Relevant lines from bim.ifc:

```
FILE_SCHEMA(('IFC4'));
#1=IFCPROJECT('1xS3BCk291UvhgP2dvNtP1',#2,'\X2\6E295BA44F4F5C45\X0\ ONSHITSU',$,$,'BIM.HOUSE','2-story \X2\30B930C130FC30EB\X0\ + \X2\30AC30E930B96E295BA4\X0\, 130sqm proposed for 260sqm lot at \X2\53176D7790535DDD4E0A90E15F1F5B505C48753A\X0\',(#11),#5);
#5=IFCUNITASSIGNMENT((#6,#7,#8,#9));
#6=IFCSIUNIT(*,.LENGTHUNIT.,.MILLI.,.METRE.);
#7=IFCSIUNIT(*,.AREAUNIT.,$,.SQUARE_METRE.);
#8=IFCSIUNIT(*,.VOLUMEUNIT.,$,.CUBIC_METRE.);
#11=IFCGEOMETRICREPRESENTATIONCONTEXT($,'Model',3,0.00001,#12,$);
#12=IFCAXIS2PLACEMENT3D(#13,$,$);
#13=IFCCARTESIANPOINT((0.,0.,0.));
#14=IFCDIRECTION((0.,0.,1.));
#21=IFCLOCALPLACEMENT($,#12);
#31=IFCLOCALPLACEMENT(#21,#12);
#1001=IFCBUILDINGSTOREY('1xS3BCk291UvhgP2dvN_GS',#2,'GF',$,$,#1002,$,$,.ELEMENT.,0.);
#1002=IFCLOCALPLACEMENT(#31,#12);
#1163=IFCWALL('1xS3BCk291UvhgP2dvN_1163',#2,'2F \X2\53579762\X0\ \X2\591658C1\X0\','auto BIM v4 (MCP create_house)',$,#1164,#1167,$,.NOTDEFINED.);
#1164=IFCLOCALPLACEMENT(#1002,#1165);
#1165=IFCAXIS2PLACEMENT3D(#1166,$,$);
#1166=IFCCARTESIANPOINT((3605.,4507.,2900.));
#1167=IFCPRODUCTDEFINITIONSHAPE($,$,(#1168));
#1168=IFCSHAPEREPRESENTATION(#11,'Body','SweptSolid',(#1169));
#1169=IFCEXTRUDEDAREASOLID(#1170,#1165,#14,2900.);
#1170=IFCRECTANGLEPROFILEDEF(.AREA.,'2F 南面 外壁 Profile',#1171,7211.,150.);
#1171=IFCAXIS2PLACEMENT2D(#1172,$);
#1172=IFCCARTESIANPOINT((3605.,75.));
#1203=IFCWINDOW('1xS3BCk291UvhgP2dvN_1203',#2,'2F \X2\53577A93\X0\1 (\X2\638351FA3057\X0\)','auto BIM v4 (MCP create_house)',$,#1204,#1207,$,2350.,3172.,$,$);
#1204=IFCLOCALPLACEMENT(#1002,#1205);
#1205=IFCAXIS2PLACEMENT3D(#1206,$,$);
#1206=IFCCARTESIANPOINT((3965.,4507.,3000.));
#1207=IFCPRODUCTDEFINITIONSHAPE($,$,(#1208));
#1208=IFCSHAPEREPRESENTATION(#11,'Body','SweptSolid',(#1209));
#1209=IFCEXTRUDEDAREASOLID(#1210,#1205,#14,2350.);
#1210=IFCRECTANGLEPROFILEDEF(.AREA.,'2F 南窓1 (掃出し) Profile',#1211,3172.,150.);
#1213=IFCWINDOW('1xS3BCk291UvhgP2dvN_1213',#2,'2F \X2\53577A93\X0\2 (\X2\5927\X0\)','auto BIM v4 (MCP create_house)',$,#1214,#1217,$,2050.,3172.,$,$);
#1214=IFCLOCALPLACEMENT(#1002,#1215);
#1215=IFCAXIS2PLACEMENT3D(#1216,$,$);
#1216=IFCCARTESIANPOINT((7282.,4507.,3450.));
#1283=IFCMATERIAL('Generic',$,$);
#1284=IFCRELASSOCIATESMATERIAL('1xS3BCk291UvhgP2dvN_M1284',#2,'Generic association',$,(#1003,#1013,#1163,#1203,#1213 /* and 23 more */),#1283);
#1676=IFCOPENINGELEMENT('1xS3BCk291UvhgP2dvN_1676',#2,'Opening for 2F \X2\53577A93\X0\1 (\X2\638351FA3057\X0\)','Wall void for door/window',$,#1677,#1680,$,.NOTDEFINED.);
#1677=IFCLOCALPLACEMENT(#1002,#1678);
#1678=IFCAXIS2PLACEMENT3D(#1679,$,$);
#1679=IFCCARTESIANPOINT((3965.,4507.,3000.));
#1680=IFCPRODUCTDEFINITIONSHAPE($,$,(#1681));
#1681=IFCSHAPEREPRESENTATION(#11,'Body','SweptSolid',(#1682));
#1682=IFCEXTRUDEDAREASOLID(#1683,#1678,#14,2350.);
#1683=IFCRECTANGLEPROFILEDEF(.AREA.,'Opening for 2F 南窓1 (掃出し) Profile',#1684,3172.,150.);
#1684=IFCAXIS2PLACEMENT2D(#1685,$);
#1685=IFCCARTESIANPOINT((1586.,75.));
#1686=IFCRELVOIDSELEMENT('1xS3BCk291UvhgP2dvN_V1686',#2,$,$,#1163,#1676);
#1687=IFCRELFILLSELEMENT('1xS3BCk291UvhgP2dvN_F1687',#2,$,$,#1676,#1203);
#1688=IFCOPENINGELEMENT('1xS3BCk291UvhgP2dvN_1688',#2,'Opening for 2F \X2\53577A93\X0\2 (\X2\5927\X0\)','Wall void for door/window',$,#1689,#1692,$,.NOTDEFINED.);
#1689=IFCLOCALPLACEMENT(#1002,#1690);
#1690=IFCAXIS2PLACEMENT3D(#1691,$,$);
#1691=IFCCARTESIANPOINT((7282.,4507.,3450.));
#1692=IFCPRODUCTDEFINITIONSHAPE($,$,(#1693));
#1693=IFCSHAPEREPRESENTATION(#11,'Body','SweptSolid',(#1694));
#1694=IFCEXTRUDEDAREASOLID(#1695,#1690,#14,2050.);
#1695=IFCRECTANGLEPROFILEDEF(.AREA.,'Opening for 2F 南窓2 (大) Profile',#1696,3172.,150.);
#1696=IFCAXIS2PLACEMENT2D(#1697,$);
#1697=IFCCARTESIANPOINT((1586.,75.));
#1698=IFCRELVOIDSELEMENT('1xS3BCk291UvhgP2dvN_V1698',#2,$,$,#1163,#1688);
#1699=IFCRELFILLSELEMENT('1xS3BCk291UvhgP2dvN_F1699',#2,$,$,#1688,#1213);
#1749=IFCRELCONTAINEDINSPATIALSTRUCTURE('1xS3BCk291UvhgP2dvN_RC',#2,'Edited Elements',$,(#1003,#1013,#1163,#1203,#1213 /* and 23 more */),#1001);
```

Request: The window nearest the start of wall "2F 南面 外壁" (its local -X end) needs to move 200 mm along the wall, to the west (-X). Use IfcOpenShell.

```python
import ifcopenshell
import ifcopenshell.api.geometry
import ifcopenshell.util.placement
import ifcopenshell.util.unit

model = ifcopenshell.open("bim.ifc")
unit_scale = ifcopenshell.util.unit.calculate_unit_scale(model)

window = model.by_guid("1xS3BCk291UvhgP2dvN_1203")
opening = window.FillsVoids[0].RelatingOpeningElement
wall = opening.VoidsElements[0].RelatingBuildingElement

wall_matrix = ifcopenshell.util.placement.get_local_placement(wall.ObjectPlacement)
shift = wall_matrix[:3, 0] * -0.2 / unit_scale
before = ifcopenshell.util.placement.get_local_placement(window.ObjectPlacement)[:3, 3].copy()

# The window is not placed relative to its opening, so move both.
for product in (opening, window):
    matrix = ifcopenshell.util.placement.get_local_placement(product.ObjectPlacement)
    matrix[:3, 3] += shift
    ifcopenshell.api.geometry.edit_object_placement(model, product=product, matrix=matrix, is_si=False)

after = ifcopenshell.util.placement.get_local_placement(window.ObjectPlacement)[:3, 3]
print("window moved by", (after - before).round(3) + 0.0)

model.write("bim_edited.ifc")
```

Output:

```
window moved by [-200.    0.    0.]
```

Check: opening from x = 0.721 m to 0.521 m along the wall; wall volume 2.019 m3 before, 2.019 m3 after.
